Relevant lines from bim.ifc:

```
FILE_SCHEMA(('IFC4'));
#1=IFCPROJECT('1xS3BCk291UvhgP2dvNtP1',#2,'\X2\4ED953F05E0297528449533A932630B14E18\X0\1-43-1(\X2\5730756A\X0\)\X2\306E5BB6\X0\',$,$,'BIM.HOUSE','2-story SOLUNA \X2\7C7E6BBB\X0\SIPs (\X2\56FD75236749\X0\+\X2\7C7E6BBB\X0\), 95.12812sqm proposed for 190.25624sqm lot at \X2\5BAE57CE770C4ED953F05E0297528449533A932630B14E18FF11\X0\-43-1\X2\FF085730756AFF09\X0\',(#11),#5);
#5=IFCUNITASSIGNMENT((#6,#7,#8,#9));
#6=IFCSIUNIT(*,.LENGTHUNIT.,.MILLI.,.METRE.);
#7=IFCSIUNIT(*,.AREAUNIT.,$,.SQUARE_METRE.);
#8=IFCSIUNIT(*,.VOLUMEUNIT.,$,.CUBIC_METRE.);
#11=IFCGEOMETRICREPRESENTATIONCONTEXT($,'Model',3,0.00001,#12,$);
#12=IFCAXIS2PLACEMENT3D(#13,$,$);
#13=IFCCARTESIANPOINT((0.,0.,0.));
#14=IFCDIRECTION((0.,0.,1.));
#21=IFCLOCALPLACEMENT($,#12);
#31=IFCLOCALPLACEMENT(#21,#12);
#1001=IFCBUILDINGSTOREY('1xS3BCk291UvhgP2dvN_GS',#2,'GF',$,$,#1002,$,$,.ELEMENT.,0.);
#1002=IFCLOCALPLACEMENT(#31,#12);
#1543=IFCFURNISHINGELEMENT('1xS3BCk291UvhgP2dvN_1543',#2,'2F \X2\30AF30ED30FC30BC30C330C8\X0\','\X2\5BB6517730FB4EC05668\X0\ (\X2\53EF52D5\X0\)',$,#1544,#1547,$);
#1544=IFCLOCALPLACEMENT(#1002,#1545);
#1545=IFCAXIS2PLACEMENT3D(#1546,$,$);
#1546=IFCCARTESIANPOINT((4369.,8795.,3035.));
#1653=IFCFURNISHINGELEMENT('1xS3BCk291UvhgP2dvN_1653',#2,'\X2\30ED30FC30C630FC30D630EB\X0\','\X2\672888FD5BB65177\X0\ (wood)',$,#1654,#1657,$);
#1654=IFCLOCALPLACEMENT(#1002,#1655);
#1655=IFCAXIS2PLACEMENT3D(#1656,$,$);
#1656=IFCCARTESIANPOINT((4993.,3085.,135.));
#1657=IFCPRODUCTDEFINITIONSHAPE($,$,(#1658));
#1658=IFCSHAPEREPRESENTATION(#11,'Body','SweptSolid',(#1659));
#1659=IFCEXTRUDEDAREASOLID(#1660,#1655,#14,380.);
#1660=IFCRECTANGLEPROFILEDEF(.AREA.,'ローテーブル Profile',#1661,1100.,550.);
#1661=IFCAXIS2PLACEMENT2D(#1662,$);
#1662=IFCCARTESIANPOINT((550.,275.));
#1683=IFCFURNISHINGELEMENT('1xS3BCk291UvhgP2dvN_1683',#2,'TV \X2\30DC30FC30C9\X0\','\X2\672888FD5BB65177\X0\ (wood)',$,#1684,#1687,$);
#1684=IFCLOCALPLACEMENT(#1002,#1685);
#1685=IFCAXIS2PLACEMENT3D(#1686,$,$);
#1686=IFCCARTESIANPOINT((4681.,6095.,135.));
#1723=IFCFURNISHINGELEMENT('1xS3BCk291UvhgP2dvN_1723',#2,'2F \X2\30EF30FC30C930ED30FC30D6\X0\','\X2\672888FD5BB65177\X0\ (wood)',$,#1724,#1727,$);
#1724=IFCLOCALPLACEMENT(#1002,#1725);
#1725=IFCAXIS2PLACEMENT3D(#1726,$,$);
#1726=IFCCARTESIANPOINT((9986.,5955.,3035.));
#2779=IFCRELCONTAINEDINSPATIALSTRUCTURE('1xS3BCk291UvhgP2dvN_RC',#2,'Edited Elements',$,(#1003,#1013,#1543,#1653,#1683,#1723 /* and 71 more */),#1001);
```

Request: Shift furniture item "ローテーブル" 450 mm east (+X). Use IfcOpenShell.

```python
import ifcopenshell
import ifcopenshell.api.geometry
import ifcopenshell.util.placement

model = ifcopenshell.open("bim.ifc")

item = model.by_guid("1xS3BCk291UvhgP2dvN_1653")
matrix = ifcopenshell.util.placement.get_local_placement(item.ObjectPlacement)
matrix[0, 3] += 450.0
ifcopenshell.api.geometry.edit_object_placement(model, product=item, matrix=matrix, is_si=False)

print(ifcopenshell.util.placement.get_local_placement(item.ObjectPlacement).round(3) + 0.0)

model.write("bim_rev.ifc")
```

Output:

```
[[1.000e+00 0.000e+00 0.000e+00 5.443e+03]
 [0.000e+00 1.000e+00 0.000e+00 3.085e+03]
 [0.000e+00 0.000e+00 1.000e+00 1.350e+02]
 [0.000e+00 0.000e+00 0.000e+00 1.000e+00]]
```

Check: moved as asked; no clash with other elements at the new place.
